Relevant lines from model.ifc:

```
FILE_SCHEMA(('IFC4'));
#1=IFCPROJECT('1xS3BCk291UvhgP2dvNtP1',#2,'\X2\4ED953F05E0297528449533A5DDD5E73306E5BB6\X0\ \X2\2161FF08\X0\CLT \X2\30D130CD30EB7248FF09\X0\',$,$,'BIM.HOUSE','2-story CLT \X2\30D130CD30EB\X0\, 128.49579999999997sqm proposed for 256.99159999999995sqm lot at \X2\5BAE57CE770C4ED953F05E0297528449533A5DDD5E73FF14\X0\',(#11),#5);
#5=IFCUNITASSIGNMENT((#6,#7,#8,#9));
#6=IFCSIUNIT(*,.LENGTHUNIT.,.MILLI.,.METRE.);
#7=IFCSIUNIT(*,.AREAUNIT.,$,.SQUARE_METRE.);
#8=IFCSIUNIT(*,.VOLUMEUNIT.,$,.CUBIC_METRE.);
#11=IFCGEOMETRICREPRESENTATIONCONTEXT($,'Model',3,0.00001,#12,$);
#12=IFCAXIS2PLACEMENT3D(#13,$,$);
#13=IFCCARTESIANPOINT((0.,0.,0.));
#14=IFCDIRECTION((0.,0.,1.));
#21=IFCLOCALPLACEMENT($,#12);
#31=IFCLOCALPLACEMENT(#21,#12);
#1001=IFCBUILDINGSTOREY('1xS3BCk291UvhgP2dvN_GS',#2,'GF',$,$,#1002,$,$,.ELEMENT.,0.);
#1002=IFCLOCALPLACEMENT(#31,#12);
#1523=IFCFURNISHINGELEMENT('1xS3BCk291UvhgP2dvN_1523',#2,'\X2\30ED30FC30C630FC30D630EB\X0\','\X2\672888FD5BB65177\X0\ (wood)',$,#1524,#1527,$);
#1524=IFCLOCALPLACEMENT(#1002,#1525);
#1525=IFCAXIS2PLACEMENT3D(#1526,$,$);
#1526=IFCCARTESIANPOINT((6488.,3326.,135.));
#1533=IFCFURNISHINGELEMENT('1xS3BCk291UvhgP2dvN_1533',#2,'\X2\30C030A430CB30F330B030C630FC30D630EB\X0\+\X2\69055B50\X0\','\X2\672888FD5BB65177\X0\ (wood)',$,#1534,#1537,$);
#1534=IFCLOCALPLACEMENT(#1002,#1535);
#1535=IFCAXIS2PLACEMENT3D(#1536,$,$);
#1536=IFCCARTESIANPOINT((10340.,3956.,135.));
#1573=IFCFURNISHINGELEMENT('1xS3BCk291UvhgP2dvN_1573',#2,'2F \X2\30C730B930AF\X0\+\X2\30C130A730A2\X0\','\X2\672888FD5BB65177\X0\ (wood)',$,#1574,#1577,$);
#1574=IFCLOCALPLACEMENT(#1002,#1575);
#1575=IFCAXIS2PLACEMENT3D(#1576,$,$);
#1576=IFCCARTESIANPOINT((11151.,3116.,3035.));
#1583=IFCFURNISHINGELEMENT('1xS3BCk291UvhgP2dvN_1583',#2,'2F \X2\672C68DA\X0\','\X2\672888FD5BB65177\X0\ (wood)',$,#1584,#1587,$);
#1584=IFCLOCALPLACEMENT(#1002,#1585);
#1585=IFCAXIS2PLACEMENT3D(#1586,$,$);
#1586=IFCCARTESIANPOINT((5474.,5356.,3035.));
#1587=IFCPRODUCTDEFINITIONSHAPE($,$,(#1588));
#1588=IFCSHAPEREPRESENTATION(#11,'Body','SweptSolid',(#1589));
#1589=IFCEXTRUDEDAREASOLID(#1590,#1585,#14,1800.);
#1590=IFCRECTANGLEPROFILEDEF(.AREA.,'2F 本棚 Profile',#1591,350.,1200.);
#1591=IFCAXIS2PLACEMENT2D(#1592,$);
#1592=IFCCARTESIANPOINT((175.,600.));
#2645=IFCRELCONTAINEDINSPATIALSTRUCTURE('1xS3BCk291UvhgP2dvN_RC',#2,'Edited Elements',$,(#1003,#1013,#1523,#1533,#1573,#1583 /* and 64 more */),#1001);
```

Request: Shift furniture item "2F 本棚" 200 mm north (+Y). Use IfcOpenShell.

```python
import ifcopenshell
import ifcopenshell.api.geometry
import ifcopenshell.util.placement

model = ifcopenshell.open("model.ifc")

item = model.by_guid("1xS3BCk291UvhgP2dvN_1583")
matrix = ifcopenshell.util.placement.get_local_placement(item.ObjectPlacement)
matrix[1, 3] += 200.0
ifcopenshell.api.geometry.edit_object_placement(model, product=item, matrix=matrix, is_si=False)

print(ifcopenshell.util.placement.get_local_placement(item.ObjectPlacement).round(3) + 0.0)

model.write("model_edited.ifc")
```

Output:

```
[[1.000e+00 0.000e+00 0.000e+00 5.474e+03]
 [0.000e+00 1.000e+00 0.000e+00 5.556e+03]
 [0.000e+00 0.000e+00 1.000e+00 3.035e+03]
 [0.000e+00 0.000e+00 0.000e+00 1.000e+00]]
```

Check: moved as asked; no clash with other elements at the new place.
